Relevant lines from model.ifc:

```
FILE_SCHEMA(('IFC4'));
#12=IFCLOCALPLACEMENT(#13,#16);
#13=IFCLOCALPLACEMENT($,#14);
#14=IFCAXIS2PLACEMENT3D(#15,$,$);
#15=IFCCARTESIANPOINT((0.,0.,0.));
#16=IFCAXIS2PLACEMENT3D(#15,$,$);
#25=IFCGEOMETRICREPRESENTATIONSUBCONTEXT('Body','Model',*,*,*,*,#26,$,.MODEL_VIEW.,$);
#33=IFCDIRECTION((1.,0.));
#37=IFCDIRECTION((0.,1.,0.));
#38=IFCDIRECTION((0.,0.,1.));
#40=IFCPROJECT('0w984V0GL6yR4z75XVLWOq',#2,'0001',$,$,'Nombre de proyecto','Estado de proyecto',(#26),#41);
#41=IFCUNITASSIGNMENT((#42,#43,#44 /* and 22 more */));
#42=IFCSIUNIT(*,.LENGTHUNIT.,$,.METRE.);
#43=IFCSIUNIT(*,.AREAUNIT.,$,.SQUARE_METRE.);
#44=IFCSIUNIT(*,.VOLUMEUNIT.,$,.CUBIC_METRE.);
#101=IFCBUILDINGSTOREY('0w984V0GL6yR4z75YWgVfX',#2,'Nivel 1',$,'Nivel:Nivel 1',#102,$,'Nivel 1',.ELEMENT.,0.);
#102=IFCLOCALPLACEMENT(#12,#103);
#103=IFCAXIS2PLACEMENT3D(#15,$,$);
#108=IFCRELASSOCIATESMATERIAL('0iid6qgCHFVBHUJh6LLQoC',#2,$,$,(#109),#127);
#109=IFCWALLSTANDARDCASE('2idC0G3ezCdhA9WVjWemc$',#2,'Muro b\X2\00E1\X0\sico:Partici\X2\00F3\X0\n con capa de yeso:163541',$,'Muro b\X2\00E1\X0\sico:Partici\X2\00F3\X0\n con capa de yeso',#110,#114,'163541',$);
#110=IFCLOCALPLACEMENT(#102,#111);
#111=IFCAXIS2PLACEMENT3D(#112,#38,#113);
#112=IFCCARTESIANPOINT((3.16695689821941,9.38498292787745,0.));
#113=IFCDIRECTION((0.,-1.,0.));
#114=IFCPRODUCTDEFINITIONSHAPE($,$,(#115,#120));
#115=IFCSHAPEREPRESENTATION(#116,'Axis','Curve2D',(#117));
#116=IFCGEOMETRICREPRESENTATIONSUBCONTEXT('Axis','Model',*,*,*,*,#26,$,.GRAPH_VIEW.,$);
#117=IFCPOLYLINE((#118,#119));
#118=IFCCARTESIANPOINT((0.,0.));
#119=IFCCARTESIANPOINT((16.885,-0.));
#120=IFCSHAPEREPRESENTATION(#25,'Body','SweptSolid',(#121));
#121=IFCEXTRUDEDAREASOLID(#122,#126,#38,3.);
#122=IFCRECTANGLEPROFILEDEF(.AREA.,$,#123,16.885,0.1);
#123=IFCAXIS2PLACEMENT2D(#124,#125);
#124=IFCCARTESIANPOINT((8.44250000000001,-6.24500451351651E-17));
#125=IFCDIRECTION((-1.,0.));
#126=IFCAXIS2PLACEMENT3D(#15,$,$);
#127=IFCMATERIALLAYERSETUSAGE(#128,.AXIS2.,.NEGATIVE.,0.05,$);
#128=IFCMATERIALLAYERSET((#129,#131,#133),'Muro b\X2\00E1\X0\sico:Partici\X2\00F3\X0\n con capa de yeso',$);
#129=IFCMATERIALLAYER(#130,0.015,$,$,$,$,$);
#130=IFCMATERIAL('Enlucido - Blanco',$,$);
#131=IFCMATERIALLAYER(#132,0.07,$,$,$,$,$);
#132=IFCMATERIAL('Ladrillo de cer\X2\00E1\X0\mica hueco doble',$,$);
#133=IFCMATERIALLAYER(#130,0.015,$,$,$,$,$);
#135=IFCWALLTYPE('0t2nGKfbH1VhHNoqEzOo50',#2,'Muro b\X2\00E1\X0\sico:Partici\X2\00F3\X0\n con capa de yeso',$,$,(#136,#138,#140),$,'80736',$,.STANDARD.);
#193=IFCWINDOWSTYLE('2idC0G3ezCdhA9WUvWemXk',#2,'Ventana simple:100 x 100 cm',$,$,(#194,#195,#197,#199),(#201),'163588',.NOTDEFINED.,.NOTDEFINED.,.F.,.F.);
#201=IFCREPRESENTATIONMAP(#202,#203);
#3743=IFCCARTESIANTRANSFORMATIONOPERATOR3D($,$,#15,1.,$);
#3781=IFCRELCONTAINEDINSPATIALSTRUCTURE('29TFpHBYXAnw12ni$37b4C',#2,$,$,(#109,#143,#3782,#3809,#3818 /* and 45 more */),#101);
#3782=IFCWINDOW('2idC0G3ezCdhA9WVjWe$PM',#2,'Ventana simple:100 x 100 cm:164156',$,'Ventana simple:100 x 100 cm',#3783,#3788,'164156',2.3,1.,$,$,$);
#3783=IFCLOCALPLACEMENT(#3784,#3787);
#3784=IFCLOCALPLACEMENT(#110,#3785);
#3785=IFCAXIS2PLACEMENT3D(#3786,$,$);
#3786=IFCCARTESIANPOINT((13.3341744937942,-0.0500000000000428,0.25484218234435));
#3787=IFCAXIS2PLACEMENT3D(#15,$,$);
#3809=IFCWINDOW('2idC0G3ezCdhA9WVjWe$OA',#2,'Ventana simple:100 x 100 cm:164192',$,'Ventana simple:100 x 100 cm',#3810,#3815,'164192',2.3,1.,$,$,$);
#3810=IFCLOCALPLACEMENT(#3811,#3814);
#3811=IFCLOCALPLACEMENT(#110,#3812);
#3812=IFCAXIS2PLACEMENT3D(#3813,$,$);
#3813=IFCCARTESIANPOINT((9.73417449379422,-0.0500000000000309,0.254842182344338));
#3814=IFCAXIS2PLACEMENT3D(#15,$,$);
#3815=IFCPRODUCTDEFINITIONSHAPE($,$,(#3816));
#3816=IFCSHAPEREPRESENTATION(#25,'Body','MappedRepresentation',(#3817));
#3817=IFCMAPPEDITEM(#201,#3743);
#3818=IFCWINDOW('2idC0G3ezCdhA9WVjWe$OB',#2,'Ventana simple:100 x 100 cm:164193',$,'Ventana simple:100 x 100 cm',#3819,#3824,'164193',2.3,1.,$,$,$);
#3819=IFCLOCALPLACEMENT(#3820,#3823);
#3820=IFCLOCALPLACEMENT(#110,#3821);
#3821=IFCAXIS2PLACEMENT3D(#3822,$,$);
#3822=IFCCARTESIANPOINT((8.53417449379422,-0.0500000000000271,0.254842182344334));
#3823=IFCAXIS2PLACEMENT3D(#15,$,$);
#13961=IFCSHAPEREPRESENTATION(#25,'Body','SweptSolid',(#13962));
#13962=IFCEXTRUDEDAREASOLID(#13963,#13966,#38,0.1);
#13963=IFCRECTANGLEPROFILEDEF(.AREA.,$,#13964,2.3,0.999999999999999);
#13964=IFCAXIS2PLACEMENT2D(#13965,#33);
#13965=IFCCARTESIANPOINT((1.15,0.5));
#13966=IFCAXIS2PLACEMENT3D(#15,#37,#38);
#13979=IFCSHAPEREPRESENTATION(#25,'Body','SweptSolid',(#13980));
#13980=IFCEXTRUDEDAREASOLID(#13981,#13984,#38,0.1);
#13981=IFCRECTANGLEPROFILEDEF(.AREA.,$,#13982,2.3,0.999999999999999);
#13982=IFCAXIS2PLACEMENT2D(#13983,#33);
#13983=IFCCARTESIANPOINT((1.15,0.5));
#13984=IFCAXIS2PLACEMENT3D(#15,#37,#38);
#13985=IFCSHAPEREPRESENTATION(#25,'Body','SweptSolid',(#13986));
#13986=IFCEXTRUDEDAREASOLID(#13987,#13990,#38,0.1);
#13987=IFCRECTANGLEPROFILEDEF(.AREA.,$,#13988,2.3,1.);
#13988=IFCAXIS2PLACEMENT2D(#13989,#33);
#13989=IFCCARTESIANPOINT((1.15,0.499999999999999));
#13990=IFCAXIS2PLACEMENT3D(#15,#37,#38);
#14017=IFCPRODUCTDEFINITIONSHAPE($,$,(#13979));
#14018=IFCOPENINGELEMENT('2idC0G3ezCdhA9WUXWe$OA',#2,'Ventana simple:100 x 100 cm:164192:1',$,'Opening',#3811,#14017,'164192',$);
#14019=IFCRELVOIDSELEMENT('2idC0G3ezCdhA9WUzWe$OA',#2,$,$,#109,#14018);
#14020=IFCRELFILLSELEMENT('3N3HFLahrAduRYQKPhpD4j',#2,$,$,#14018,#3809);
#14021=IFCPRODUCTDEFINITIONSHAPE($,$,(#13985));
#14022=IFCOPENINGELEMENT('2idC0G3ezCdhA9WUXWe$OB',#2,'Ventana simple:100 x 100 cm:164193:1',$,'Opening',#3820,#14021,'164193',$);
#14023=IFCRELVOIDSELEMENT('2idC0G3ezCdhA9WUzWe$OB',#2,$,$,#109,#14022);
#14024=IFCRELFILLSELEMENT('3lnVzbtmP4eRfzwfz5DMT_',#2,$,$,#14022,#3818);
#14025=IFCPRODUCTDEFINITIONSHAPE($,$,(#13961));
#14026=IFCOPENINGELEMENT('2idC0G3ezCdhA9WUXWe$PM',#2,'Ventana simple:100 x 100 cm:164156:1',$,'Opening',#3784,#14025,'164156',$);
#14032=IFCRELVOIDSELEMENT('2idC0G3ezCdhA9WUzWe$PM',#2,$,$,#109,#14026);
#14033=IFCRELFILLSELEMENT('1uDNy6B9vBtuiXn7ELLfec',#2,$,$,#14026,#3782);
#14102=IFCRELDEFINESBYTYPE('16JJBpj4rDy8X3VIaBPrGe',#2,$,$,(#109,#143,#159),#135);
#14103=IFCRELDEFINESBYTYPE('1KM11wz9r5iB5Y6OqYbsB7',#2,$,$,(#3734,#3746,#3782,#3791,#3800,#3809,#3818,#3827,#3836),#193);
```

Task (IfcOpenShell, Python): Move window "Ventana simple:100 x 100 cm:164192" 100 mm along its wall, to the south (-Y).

```python
import ifcopenshell
import ifcopenshell.api.geometry
import ifcopenshell.util.placement
import ifcopenshell.util.unit

model = ifcopenshell.open("model.ifc")
unit_scale = ifcopenshell.util.unit.calculate_unit_scale(model)

window = model.by_id(3809)
opening = window.FillsVoids[0].RelatingOpeningElement
wall = opening.VoidsElements[0].RelatingBuildingElement

wall_matrix = ifcopenshell.util.placement.get_local_placement(wall.ObjectPlacement)
shift = wall_matrix[:3, 0] * 0.1 / unit_scale
before = ifcopenshell.util.placement.get_local_placement(window.ObjectPlacement)[:3, 3].copy()

# The window is placed relative to its opening, so it follows when the opening moves.
matrix = ifcopenshell.util.placement.get_local_placement(opening.ObjectPlacement)
matrix[:3, 3] += shift
ifcopenshell.api.geometry.edit_object_placement(
    model, product=opening, matrix=matrix, is_si=False, should_transform_children=True
)

after = ifcopenshell.util.placement.get_local_placement(window.ObjectPlacement)[:3, 3]
print("window moved by", (after - before).round(3) + 0.0)

model.write("model-out.ifc")
```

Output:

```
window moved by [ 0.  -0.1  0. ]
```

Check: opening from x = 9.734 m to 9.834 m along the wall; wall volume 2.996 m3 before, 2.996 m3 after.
